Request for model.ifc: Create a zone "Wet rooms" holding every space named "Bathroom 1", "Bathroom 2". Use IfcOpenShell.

First a look at what the model holds.

```python
import ifcopenshell

model = ifcopenshell.open("model.ifc")
print(model.schema)
seen = {}
for space in model.by_type("IfcSpace"):
    seen[space.LongName] = seen.get(space.LongName, 0) + 1
for name, count in sorted(seen.items(), key=str):
    print(count, "x", name)
print("zones:", [z.Name for z in model.by_type("IfcZone")][:20])
```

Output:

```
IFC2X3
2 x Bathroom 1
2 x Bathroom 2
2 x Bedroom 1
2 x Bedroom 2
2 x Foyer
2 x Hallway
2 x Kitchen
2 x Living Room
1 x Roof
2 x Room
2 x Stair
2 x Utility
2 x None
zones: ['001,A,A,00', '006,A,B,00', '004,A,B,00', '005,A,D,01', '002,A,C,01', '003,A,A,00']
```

```python
import ifcopenshell
import ifcopenshell.api.group
import ifcopenshell.api.root

model = ifcopenshell.open("model.ifc")

names = {"Bathroom 1", "Bathroom 2"}
spaces = [s for s in model.by_type("IfcSpace") if s.LongName in names]

zone = ifcopenshell.api.root.create_entity(model, ifc_class="IfcZone", name="Wet rooms")
ifcopenshell.api.group.assign_group(model, products=spaces, group=zone)
print(len(spaces), "spaces in", zone.Name)

model.write("model_v2.ifc")
```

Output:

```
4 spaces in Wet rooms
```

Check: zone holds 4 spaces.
